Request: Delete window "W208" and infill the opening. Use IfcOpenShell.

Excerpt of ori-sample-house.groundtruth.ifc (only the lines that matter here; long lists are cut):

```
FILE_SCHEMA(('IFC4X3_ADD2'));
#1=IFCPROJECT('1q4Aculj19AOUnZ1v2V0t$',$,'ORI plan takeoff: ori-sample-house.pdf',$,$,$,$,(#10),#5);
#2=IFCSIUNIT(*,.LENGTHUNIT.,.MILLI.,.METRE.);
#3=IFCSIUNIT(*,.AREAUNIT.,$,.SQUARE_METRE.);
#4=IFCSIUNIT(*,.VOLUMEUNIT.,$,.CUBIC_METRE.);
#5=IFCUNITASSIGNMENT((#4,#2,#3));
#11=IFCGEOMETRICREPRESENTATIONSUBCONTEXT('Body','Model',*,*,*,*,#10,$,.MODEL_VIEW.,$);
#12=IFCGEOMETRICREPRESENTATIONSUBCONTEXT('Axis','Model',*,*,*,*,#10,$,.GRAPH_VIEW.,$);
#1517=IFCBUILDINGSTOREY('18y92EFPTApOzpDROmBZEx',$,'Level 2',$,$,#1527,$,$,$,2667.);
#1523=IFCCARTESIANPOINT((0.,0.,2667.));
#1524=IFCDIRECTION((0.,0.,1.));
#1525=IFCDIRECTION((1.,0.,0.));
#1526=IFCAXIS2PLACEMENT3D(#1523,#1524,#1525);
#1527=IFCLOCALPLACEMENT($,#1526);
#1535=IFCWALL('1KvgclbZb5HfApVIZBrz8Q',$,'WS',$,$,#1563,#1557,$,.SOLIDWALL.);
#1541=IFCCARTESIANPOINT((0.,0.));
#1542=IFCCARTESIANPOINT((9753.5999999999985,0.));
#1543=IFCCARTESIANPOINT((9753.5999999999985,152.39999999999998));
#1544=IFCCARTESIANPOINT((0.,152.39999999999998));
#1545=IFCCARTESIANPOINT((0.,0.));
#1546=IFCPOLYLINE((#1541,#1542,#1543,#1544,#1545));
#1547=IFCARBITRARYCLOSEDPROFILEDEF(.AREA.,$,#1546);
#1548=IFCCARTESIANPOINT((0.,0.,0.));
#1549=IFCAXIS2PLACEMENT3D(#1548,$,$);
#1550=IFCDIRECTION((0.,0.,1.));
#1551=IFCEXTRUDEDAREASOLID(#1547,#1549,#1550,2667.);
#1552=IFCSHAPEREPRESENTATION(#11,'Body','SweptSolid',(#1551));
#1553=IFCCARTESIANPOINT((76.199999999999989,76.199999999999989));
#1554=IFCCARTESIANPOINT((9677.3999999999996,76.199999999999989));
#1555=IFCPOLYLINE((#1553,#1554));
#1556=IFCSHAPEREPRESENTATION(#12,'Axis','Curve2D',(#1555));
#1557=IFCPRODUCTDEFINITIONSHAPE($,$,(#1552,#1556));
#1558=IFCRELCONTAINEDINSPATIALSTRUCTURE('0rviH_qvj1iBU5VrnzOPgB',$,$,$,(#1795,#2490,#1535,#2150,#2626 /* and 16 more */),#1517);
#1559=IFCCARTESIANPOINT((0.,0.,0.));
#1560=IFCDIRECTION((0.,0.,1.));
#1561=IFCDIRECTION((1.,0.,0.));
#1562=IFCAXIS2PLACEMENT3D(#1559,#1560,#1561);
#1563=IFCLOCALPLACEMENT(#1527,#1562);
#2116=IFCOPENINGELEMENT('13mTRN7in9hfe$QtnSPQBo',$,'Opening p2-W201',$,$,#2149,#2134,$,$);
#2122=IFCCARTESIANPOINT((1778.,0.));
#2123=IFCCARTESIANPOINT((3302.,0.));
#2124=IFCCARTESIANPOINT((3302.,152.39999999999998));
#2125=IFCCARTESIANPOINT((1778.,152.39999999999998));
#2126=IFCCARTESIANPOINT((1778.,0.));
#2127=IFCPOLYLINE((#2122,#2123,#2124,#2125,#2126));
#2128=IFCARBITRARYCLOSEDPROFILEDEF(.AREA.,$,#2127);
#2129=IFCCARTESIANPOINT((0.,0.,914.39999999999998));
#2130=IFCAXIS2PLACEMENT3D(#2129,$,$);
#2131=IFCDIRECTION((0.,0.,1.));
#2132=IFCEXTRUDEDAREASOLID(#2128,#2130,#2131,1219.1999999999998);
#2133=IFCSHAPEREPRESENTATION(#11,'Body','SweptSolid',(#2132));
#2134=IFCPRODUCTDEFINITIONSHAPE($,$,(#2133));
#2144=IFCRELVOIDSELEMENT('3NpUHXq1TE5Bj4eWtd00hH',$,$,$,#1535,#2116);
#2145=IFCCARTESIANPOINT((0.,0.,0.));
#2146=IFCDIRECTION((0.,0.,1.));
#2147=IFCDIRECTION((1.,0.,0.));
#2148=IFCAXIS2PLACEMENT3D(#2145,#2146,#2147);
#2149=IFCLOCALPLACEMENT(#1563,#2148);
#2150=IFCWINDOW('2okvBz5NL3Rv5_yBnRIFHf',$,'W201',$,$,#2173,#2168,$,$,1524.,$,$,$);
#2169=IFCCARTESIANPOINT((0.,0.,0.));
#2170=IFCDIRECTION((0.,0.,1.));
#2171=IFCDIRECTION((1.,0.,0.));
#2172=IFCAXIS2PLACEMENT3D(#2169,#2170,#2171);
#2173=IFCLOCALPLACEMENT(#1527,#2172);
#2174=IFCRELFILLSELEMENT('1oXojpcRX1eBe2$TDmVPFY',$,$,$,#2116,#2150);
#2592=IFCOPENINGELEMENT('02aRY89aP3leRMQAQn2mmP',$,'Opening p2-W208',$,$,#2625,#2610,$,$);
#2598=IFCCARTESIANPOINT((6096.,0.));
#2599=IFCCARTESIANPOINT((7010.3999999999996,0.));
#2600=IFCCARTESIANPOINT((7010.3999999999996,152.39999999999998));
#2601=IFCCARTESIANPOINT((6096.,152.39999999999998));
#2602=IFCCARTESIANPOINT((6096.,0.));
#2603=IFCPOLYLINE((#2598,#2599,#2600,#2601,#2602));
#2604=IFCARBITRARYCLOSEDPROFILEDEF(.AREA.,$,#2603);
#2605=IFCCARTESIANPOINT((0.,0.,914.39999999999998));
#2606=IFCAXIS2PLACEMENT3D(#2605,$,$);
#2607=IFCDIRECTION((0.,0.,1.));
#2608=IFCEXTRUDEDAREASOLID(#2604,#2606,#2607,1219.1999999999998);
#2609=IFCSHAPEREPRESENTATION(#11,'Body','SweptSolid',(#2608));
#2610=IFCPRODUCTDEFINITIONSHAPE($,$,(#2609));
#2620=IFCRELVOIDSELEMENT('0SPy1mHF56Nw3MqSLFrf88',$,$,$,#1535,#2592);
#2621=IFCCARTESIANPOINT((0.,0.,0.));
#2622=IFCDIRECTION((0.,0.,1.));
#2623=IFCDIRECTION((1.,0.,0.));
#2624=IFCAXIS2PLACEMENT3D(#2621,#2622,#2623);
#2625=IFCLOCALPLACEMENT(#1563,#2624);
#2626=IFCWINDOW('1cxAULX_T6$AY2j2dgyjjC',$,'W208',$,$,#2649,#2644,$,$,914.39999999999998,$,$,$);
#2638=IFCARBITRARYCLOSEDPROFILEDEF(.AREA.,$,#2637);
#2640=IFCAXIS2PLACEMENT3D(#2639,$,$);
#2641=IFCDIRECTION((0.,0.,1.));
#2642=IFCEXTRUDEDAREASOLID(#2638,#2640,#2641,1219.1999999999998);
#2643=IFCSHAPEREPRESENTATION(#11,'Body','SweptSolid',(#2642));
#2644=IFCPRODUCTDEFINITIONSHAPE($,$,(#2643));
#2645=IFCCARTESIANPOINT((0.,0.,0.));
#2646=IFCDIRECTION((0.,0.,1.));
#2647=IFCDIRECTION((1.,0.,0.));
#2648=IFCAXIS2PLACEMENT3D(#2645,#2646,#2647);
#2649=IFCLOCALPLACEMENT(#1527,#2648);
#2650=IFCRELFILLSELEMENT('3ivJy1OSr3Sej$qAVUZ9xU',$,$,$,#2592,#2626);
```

```python
import ifcopenshell
import ifcopenshell.api.feature
import ifcopenshell.api.root
import ifcopenshell.geom
import ifcopenshell.util.shape

model = ifcopenshell.open("ori-sample-house.groundtruth.ifc")
settings = ifcopenshell.geom.settings()


def volume(element):
    """Net volume in cubic metres, openings subtracted."""
    shape = ifcopenshell.geom.create_shape(settings, element)
    return ifcopenshell.util.shape.get_volume(shape.geometry)


window = model.by_guid("1cxAULX_T6$AY2j2dgyjjC")
opening = window.FillsVoids[0].RelatingOpeningElement
wall = opening.VoidsElements[0].RelatingBuildingElement
before = volume(wall)

ifcopenshell.api.root.remove_product(model, product=window)
ifcopenshell.api.feature.remove_feature(model, feature=opening)

after = volume(wall)

print(f"wall volume {before:.3f} -> {after:.3f} m3")

model.write("ori-sample-house.groundtruth_edited.ifc")
```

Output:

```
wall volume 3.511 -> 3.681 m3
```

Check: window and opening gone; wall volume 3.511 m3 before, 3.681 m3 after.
